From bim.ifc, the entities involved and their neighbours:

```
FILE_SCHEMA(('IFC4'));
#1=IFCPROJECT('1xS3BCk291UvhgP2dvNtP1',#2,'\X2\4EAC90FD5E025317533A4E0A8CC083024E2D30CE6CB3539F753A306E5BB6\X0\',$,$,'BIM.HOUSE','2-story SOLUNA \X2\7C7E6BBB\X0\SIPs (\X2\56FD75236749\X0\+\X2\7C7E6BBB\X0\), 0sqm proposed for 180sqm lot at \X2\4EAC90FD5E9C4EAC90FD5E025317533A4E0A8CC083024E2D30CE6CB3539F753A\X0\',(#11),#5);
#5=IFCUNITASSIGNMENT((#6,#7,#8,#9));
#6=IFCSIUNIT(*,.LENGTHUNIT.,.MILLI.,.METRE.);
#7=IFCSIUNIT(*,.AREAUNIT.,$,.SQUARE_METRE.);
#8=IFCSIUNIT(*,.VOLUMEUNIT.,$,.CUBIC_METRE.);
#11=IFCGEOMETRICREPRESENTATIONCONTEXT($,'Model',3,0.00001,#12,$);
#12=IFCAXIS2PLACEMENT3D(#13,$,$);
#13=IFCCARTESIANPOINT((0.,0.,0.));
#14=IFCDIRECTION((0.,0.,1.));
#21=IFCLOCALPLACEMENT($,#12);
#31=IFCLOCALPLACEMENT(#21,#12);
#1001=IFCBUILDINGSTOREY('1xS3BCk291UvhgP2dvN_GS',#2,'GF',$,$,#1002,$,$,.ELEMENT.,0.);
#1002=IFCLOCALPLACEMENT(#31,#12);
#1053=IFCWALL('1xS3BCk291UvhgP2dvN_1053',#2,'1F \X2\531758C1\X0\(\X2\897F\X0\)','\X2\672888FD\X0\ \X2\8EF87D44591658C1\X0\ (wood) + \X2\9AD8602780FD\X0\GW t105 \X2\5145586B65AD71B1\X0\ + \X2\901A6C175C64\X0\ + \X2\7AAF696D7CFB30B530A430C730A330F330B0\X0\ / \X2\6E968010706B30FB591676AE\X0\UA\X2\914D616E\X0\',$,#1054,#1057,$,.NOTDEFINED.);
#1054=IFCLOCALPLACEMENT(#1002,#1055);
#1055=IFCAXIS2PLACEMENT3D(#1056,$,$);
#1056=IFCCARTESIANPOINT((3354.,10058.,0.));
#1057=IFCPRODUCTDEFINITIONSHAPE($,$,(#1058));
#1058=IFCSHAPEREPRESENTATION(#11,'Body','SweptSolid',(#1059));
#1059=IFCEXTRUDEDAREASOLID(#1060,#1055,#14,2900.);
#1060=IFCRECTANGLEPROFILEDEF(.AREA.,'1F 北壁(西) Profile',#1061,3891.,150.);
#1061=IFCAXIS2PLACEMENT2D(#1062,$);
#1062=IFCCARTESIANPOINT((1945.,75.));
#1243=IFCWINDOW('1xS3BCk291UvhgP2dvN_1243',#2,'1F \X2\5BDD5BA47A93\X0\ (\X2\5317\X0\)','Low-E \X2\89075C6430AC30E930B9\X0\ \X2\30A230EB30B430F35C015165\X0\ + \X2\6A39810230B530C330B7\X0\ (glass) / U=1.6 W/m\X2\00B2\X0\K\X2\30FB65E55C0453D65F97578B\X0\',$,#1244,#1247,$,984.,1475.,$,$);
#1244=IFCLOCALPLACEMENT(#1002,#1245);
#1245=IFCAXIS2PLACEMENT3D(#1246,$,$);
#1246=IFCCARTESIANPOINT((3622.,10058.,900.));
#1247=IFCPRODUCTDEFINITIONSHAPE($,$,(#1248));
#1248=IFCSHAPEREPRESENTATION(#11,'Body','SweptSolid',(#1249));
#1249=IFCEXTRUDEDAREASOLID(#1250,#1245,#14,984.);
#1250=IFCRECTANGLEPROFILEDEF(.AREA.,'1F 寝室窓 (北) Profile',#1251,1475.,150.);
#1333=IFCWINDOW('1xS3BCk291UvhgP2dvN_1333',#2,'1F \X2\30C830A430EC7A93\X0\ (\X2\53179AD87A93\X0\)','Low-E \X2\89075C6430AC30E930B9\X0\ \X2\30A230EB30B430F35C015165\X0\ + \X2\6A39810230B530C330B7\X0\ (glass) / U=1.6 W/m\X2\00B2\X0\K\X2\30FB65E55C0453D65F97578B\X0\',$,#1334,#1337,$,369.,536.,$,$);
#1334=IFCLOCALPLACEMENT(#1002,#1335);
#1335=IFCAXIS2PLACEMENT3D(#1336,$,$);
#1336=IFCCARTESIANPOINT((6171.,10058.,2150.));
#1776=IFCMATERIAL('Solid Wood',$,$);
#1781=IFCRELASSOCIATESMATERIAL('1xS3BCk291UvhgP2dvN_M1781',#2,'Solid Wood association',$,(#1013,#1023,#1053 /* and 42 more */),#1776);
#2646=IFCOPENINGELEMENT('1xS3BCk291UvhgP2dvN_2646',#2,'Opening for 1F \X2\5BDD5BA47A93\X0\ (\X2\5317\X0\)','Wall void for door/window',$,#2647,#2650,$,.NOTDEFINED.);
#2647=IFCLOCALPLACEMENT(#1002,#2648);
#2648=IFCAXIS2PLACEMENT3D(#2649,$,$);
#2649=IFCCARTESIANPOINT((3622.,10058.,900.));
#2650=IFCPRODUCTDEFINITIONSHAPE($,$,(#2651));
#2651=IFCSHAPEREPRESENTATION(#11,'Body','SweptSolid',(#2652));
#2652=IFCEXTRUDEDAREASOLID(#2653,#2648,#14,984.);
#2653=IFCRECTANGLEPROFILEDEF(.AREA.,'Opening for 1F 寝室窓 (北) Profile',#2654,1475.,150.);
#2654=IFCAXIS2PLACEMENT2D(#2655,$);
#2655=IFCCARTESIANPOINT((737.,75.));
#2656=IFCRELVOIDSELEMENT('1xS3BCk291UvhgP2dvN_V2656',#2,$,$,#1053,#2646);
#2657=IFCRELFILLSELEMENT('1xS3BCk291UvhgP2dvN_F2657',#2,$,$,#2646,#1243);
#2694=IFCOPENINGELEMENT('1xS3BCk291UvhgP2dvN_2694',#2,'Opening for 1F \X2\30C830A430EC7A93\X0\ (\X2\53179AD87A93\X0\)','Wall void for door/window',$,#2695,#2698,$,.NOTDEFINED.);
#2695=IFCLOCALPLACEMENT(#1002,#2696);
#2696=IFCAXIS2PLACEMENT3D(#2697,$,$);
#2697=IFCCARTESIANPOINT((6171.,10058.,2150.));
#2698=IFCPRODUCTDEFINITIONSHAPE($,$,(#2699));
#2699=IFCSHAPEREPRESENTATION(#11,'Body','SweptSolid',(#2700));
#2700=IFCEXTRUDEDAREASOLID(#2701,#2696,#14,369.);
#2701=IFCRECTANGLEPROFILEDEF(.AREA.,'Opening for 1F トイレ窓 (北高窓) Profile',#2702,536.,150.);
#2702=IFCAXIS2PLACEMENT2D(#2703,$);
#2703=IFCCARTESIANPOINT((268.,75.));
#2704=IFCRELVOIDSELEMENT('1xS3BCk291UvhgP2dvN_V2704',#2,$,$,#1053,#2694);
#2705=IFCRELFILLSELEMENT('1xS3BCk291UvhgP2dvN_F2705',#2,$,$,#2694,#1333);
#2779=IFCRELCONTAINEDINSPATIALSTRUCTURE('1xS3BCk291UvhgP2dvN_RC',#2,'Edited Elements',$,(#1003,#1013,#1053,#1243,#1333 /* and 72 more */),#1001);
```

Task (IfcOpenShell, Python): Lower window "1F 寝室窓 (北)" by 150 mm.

```python
import numpy as np
import ifcopenshell
import ifcopenshell.api.geometry
import ifcopenshell.util.placement
import ifcopenshell.util.unit

model = ifcopenshell.open("bim.ifc")
unit_scale = ifcopenshell.util.unit.calculate_unit_scale(model)

window = model.by_guid("1xS3BCk291UvhgP2dvN_1243")
opening = window.FillsVoids[0].RelatingOpeningElement
dz = -0.15 / unit_scale

shift = np.array([0.0, 0.0, dz])
# The window is not placed relative to its opening, so move both.
for product in (opening, window):
    matrix = ifcopenshell.util.placement.get_local_placement(product.ObjectPlacement)
    matrix[:3, 3] += shift
    ifcopenshell.api.geometry.edit_object_placement(model, product=product, matrix=matrix, is_si=False)

print(f"moved by {dz * unit_scale:+.3f} m")

model.write("bim_rev.ifc")
```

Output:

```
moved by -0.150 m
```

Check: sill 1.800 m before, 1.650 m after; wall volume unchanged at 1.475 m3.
